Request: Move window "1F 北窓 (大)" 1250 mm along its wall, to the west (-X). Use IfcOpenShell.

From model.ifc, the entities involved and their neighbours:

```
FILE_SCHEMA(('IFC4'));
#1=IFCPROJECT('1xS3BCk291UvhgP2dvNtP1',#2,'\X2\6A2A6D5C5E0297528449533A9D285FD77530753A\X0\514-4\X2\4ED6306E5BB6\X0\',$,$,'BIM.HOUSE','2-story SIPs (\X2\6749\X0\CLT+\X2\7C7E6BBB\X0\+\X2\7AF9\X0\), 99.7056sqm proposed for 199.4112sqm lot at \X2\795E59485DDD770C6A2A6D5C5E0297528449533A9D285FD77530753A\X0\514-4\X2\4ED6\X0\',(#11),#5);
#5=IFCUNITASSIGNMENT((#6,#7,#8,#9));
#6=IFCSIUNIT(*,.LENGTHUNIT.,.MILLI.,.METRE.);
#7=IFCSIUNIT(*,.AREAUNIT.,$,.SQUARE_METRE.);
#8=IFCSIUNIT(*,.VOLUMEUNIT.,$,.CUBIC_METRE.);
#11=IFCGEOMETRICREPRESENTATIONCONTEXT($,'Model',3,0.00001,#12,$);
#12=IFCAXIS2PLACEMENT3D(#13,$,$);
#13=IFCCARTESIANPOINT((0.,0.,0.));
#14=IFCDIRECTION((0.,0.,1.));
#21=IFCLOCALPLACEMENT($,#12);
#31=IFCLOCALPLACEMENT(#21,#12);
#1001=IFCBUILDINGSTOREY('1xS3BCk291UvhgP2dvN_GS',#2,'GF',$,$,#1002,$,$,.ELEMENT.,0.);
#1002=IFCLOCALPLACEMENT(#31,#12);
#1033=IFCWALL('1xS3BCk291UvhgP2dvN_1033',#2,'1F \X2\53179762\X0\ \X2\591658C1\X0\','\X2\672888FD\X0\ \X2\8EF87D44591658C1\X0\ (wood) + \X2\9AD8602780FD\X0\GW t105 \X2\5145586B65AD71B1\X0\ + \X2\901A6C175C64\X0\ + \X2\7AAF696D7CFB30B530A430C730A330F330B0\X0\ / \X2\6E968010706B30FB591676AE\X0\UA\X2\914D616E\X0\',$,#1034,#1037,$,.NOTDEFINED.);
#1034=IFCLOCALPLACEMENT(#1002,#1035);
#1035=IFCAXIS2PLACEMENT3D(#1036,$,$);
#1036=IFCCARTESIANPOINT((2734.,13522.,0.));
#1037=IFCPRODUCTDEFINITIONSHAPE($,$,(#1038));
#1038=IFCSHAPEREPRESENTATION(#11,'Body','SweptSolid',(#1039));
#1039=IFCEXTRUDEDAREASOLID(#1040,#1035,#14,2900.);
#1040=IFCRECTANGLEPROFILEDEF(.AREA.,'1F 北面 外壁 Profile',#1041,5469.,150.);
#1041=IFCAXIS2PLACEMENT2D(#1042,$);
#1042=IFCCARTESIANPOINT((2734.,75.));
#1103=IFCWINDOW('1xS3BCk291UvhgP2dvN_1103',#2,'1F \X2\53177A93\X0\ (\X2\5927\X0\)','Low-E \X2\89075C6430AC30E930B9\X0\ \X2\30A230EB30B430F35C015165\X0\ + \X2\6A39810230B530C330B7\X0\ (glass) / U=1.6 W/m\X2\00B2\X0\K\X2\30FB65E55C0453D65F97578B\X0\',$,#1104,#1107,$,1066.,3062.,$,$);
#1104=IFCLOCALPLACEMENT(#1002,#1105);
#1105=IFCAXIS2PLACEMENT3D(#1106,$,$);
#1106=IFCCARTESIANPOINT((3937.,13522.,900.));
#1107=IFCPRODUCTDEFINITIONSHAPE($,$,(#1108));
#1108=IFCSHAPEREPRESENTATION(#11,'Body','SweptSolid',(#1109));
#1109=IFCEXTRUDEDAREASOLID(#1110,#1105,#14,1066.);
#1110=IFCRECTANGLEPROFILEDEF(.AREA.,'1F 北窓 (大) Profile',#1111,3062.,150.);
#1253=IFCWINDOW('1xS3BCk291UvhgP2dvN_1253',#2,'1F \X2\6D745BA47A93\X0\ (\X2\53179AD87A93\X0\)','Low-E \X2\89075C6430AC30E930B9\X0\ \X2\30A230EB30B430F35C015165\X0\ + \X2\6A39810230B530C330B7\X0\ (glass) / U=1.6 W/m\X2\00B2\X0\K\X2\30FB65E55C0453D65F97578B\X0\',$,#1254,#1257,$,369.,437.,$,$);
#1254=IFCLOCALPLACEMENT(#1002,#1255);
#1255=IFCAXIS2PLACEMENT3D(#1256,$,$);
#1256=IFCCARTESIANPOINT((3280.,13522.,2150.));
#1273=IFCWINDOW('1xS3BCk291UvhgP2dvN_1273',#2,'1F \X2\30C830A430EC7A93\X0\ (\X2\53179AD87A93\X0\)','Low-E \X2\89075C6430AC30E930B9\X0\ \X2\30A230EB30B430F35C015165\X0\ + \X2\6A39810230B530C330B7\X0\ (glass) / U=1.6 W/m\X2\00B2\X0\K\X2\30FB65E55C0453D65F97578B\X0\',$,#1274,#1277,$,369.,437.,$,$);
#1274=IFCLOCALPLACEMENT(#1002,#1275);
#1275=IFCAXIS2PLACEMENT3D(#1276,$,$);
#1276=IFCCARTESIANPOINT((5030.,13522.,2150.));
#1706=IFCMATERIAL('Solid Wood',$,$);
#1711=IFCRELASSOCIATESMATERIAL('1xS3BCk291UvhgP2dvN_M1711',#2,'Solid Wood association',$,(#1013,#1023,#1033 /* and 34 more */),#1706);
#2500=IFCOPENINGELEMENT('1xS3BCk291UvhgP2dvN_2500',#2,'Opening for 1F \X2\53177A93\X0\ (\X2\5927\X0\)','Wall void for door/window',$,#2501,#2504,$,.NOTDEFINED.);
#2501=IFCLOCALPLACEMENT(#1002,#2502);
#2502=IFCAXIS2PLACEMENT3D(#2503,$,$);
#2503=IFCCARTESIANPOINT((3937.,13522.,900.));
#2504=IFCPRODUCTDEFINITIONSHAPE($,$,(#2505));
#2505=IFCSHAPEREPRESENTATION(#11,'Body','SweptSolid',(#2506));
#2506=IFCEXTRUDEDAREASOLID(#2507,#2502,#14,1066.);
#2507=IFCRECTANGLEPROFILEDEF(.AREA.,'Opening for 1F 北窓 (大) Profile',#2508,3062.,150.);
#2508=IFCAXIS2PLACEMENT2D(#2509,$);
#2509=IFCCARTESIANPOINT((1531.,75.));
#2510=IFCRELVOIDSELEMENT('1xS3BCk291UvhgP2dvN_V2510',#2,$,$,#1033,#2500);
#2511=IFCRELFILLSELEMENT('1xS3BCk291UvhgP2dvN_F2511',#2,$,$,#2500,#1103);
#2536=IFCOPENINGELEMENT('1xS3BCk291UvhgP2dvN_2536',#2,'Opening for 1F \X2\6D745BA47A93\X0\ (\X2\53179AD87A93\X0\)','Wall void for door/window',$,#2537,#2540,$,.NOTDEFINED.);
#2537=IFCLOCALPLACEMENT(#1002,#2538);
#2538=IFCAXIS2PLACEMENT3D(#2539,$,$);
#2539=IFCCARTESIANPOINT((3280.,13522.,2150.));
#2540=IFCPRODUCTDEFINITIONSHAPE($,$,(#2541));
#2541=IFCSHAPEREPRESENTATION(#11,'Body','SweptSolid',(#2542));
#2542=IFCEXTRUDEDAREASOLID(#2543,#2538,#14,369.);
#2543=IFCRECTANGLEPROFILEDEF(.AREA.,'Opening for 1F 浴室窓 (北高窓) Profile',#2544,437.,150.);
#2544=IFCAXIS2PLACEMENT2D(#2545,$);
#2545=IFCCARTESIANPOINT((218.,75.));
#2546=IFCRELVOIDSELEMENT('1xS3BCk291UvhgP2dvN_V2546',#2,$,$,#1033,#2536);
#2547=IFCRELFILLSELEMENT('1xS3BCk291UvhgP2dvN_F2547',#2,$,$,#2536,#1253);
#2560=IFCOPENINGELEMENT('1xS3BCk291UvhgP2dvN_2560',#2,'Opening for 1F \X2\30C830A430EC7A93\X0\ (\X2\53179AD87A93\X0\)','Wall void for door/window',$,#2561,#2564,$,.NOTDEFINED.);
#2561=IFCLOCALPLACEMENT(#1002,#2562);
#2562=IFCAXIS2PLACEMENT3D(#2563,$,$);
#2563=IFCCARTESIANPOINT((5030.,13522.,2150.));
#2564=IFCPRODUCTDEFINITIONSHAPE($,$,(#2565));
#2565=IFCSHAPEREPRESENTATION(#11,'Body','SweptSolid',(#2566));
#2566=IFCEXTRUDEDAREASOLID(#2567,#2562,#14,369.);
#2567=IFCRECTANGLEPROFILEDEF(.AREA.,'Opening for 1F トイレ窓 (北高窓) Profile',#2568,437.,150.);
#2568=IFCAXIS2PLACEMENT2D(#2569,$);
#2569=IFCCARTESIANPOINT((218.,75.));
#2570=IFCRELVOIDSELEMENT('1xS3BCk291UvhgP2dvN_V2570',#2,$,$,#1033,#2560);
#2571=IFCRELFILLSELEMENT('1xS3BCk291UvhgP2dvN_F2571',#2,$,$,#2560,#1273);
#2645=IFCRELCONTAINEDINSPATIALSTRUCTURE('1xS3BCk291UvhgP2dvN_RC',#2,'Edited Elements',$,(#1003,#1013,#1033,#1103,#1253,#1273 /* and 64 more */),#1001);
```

```python
import ifcopenshell
import ifcopenshell.api.geometry
import ifcopenshell.util.placement

model = ifcopenshell.open("model.ifc")

window = model.by_guid("1xS3BCk291UvhgP2dvN_1103")
opening = window.FillsVoids[0].RelatingOpeningElement
wall = opening.VoidsElements[0].RelatingBuildingElement

wall_matrix = ifcopenshell.util.placement.get_local_placement(wall.ObjectPlacement)
shift = wall_matrix[:3, 0] * -1250.0
before = ifcopenshell.util.placement.get_local_placement(window.ObjectPlacement)[:3, 3].copy()

# The window is not placed relative to its opening, so move both.
for product in (opening, window):
    matrix = ifcopenshell.util.placement.get_local_placement(product.ObjectPlacement)
    matrix[:3, 3] += shift
    ifcopenshell.api.geometry.edit_object_placement(model, product=product, matrix=matrix, is_si=False)

after = ifcopenshell.util.placement.get_local_placement(window.ObjectPlacement)[:3, 3]
print("window moved by", (after - before).round(3) + 0.0)

model.write("model_v2.ifc")
```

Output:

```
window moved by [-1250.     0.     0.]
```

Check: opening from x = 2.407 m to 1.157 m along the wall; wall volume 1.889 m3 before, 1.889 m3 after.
